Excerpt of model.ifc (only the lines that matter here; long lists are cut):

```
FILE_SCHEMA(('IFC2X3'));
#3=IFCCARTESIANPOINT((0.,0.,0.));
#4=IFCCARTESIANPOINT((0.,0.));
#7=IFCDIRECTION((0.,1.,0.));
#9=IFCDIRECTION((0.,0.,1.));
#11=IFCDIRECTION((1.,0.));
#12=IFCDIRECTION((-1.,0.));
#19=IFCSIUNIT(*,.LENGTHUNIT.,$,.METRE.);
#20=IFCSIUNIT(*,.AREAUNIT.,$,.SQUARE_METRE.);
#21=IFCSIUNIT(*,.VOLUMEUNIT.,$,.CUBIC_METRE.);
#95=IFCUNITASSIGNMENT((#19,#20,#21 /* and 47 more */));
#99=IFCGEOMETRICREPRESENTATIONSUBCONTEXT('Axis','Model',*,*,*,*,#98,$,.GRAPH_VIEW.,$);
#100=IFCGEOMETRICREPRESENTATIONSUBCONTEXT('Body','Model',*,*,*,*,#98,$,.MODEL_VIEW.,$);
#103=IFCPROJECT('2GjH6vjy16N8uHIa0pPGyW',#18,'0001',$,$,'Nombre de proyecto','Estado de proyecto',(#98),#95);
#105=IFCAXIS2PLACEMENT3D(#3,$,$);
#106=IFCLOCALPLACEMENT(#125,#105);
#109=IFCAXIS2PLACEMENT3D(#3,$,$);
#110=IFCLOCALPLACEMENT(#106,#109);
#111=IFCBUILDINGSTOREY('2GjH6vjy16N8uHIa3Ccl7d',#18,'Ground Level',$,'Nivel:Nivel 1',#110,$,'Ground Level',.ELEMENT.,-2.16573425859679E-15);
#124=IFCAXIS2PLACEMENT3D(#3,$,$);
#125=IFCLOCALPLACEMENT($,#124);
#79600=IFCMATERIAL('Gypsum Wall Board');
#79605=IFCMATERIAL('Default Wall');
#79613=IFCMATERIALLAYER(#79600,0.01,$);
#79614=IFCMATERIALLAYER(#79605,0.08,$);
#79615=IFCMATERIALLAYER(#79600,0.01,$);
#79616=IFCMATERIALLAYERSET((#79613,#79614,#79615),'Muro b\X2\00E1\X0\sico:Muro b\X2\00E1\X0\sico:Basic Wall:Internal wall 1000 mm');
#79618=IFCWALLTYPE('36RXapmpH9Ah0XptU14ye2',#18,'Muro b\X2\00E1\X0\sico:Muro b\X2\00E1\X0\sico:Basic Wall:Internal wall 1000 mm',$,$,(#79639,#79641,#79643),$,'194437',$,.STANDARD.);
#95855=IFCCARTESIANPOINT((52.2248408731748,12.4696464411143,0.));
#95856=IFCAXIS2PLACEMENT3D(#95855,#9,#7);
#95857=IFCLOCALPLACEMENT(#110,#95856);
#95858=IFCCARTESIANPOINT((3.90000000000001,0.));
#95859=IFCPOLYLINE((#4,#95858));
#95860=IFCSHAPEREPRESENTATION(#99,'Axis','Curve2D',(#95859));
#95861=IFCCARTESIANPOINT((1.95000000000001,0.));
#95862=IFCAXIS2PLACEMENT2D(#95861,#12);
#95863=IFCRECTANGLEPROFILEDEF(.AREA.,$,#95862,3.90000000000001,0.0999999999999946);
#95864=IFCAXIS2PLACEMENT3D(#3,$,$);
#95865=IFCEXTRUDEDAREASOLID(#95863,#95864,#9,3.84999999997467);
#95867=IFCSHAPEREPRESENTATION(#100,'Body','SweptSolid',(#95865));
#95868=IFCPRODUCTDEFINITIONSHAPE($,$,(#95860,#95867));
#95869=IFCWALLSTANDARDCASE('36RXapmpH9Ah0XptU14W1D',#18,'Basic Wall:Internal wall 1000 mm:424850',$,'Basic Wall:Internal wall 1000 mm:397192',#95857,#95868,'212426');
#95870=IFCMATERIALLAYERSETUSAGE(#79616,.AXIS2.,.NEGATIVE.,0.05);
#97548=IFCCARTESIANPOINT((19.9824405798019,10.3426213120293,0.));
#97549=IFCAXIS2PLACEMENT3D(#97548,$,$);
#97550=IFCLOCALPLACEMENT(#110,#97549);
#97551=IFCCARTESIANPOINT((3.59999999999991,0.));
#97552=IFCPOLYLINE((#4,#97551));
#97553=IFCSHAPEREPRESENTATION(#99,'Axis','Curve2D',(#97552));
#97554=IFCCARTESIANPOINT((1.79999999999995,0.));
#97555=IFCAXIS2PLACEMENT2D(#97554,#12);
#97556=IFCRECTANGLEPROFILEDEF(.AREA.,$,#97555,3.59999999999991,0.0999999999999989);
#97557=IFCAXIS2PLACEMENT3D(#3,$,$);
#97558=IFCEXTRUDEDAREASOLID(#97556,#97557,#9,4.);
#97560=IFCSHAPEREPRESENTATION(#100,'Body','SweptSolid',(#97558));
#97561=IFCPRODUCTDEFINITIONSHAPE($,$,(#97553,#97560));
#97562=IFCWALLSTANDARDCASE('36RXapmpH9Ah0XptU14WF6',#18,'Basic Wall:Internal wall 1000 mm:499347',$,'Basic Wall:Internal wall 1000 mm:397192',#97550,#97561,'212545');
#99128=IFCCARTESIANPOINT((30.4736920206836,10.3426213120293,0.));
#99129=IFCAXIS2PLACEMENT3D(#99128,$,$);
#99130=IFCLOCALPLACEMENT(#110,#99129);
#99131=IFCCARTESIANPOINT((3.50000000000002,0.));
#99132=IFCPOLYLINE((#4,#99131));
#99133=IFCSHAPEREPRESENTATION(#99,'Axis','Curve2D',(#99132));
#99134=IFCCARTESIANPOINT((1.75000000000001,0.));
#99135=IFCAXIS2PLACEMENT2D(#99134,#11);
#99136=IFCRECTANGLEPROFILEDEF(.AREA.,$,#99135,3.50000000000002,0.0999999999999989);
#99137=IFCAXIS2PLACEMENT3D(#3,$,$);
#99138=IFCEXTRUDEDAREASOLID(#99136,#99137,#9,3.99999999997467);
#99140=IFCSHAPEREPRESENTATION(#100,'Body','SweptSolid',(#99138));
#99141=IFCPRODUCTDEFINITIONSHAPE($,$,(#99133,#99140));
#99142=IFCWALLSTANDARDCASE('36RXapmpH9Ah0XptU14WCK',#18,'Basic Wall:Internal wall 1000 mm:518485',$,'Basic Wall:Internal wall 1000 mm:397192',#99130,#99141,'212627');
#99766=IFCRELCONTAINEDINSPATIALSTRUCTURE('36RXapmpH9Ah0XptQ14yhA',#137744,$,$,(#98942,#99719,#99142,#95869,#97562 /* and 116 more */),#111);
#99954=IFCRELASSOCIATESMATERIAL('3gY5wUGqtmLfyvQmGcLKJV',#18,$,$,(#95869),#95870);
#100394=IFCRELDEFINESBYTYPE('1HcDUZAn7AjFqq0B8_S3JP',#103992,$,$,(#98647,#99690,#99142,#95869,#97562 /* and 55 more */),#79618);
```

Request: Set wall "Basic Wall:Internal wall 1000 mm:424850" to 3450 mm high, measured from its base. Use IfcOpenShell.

```python
import ifcopenshell
import ifcopenshell.geom
import ifcopenshell.util.representation
import ifcopenshell.util.shape

model = ifcopenshell.open("model.ifc")
settings = ifcopenshell.geom.settings()


def volume(element):
    """Net volume in cubic metres, openings subtracted."""
    shape = ifcopenshell.geom.create_shape(settings, element)
    return ifcopenshell.util.shape.get_volume(shape.geometry)


wall = model.by_guid("36RXapmpH9Ah0XptU14W1D")
before = volume(wall)

body = ifcopenshell.util.representation.get_representation(wall, "Model", "Body")
solid = body.Items[0]
old_height = solid.Depth
solid.Depth = 3.45
after = volume(wall)

print(f"height {old_height:g} -> {solid.Depth:g}, volume {before:.3f} -> {after:.3f} m3")

model.write("model_edited.ifc")
```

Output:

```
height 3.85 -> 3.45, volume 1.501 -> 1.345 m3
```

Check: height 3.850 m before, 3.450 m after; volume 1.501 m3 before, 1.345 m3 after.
